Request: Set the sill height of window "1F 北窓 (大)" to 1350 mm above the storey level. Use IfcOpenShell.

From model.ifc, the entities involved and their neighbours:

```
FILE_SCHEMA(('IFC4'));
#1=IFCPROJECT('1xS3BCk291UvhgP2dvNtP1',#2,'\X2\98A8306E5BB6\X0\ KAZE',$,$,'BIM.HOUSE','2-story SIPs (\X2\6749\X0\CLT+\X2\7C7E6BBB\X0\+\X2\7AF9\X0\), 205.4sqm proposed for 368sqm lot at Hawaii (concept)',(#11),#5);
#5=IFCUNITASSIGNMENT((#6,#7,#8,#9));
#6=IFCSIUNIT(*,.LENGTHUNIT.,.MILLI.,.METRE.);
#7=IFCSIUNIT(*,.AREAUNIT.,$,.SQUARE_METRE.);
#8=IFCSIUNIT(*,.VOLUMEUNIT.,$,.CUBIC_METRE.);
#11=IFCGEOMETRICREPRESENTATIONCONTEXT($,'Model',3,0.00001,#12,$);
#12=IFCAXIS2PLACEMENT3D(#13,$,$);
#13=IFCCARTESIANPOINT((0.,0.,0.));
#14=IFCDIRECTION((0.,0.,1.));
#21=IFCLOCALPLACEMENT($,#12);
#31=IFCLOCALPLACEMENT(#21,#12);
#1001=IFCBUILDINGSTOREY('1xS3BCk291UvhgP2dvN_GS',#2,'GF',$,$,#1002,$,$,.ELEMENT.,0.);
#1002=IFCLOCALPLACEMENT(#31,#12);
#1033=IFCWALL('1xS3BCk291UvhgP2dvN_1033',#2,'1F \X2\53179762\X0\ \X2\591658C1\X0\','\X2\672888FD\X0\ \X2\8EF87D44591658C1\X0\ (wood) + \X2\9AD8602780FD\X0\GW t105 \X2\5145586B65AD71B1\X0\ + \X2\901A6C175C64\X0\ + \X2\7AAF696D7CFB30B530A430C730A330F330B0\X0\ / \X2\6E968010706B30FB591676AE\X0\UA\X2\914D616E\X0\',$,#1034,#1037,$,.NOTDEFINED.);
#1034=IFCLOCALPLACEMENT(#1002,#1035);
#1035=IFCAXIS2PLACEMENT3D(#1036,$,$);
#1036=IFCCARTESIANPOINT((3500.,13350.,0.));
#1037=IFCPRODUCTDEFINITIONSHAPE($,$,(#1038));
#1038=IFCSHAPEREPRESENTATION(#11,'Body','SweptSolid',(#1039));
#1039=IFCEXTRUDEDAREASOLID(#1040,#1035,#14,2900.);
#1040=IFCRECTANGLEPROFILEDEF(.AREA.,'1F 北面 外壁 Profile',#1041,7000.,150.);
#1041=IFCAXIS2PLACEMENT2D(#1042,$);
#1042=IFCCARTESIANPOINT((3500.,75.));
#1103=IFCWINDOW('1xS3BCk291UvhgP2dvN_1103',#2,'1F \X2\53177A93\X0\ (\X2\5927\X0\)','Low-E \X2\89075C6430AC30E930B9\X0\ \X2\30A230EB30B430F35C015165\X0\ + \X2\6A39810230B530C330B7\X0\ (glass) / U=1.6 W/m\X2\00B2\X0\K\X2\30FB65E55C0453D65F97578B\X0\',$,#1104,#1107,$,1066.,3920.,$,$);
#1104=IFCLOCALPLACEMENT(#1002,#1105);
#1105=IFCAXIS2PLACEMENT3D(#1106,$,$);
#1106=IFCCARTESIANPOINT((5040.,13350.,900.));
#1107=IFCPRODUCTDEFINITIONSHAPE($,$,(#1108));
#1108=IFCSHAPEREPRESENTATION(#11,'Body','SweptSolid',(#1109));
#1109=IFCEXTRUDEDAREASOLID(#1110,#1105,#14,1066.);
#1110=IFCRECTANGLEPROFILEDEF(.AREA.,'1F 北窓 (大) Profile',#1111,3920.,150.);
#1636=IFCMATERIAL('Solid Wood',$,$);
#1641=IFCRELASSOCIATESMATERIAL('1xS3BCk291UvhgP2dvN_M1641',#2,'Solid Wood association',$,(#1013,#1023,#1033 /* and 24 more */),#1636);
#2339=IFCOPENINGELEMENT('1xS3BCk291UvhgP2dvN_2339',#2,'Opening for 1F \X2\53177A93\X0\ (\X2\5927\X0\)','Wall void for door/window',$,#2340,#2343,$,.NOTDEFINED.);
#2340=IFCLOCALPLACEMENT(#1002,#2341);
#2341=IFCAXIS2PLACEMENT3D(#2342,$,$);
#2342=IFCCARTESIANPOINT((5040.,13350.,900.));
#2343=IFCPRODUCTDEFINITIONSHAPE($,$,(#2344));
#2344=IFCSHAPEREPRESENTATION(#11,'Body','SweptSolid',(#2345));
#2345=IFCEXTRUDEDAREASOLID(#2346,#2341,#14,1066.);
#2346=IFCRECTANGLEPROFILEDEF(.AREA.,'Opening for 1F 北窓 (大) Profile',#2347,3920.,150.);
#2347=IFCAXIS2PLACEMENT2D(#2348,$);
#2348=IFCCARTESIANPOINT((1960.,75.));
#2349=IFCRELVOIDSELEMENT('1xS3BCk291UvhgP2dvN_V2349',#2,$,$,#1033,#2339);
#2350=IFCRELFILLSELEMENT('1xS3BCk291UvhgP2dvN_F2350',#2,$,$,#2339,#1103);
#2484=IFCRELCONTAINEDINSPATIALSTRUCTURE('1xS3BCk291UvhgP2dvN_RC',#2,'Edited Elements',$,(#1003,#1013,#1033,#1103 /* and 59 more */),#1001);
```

```python
import numpy as np
import ifcopenshell
import ifcopenshell.api.geometry
import ifcopenshell.geom
import ifcopenshell.util.element
import ifcopenshell.util.placement
import ifcopenshell.util.shape
import ifcopenshell.util.unit

model = ifcopenshell.open("model.ifc")
unit_scale = ifcopenshell.util.unit.calculate_unit_scale(model)

window = model.by_id(1103)
opening = window.FillsVoids[0].RelatingOpeningElement
storey = ifcopenshell.util.element.get_container(window, ifc_class="IfcBuildingStorey")
level = ifcopenshell.util.placement.get_local_placement(storey.ObjectPlacement)[2, 3]

# The opening's origin need not be at the sill, so measure its lowest point.
shape = ifcopenshell.geom.create_shape(ifcopenshell.geom.settings(), opening)
bottom = ifcopenshell.util.shape.get_shape_bottom_elevation(shape, shape.geometry) / unit_scale
dz = level + 1.35 / unit_scale - bottom

shift = np.array([0.0, 0.0, dz])
# The window is not placed relative to its opening, so move both.
for product in (opening, window):
    matrix = ifcopenshell.util.placement.get_local_placement(product.ObjectPlacement)
    matrix[:3, 3] += shift
    ifcopenshell.api.geometry.edit_object_placement(model, product=product, matrix=matrix, is_si=False)

print(f"moved by {dz * unit_scale:+.3f} m")

model.write("model_edited.ifc")
```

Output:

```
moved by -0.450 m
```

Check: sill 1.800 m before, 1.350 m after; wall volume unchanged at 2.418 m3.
